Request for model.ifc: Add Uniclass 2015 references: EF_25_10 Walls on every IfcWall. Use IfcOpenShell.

First a look at what the model holds.

```python
import ifcopenshell

model = ifcopenshell.open("model.ifc")
print(model.schema)
print("classifications:", [c.Name for c in model.by_type("IfcClassification")])
for ifc_class in ("IfcDoor", "IfcRoof", "IfcStair", "IfcWall", "IfcWindow"):
    print(ifc_class, len(model.by_type(ifc_class)))
```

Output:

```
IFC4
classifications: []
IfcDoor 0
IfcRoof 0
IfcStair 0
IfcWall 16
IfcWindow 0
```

```python
import ifcopenshell
import ifcopenshell.api.classification

model = ifcopenshell.open("model.ifc")

system = ifcopenshell.api.classification.add_classification(model, classification="Uniclass 2015")

codes = {
    "IfcWall": ("EF_25_10", "Walls"),
}
for ifc_class, (code, name) in codes.items():
    products = model.by_type(ifc_class)
    ifcopenshell.api.classification.add_reference(
        model, products=products, classification=system, identification=code, name=name
    )
    print(code, len(products))

model.write("model_edited.ifc")
```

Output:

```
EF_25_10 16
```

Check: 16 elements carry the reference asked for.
